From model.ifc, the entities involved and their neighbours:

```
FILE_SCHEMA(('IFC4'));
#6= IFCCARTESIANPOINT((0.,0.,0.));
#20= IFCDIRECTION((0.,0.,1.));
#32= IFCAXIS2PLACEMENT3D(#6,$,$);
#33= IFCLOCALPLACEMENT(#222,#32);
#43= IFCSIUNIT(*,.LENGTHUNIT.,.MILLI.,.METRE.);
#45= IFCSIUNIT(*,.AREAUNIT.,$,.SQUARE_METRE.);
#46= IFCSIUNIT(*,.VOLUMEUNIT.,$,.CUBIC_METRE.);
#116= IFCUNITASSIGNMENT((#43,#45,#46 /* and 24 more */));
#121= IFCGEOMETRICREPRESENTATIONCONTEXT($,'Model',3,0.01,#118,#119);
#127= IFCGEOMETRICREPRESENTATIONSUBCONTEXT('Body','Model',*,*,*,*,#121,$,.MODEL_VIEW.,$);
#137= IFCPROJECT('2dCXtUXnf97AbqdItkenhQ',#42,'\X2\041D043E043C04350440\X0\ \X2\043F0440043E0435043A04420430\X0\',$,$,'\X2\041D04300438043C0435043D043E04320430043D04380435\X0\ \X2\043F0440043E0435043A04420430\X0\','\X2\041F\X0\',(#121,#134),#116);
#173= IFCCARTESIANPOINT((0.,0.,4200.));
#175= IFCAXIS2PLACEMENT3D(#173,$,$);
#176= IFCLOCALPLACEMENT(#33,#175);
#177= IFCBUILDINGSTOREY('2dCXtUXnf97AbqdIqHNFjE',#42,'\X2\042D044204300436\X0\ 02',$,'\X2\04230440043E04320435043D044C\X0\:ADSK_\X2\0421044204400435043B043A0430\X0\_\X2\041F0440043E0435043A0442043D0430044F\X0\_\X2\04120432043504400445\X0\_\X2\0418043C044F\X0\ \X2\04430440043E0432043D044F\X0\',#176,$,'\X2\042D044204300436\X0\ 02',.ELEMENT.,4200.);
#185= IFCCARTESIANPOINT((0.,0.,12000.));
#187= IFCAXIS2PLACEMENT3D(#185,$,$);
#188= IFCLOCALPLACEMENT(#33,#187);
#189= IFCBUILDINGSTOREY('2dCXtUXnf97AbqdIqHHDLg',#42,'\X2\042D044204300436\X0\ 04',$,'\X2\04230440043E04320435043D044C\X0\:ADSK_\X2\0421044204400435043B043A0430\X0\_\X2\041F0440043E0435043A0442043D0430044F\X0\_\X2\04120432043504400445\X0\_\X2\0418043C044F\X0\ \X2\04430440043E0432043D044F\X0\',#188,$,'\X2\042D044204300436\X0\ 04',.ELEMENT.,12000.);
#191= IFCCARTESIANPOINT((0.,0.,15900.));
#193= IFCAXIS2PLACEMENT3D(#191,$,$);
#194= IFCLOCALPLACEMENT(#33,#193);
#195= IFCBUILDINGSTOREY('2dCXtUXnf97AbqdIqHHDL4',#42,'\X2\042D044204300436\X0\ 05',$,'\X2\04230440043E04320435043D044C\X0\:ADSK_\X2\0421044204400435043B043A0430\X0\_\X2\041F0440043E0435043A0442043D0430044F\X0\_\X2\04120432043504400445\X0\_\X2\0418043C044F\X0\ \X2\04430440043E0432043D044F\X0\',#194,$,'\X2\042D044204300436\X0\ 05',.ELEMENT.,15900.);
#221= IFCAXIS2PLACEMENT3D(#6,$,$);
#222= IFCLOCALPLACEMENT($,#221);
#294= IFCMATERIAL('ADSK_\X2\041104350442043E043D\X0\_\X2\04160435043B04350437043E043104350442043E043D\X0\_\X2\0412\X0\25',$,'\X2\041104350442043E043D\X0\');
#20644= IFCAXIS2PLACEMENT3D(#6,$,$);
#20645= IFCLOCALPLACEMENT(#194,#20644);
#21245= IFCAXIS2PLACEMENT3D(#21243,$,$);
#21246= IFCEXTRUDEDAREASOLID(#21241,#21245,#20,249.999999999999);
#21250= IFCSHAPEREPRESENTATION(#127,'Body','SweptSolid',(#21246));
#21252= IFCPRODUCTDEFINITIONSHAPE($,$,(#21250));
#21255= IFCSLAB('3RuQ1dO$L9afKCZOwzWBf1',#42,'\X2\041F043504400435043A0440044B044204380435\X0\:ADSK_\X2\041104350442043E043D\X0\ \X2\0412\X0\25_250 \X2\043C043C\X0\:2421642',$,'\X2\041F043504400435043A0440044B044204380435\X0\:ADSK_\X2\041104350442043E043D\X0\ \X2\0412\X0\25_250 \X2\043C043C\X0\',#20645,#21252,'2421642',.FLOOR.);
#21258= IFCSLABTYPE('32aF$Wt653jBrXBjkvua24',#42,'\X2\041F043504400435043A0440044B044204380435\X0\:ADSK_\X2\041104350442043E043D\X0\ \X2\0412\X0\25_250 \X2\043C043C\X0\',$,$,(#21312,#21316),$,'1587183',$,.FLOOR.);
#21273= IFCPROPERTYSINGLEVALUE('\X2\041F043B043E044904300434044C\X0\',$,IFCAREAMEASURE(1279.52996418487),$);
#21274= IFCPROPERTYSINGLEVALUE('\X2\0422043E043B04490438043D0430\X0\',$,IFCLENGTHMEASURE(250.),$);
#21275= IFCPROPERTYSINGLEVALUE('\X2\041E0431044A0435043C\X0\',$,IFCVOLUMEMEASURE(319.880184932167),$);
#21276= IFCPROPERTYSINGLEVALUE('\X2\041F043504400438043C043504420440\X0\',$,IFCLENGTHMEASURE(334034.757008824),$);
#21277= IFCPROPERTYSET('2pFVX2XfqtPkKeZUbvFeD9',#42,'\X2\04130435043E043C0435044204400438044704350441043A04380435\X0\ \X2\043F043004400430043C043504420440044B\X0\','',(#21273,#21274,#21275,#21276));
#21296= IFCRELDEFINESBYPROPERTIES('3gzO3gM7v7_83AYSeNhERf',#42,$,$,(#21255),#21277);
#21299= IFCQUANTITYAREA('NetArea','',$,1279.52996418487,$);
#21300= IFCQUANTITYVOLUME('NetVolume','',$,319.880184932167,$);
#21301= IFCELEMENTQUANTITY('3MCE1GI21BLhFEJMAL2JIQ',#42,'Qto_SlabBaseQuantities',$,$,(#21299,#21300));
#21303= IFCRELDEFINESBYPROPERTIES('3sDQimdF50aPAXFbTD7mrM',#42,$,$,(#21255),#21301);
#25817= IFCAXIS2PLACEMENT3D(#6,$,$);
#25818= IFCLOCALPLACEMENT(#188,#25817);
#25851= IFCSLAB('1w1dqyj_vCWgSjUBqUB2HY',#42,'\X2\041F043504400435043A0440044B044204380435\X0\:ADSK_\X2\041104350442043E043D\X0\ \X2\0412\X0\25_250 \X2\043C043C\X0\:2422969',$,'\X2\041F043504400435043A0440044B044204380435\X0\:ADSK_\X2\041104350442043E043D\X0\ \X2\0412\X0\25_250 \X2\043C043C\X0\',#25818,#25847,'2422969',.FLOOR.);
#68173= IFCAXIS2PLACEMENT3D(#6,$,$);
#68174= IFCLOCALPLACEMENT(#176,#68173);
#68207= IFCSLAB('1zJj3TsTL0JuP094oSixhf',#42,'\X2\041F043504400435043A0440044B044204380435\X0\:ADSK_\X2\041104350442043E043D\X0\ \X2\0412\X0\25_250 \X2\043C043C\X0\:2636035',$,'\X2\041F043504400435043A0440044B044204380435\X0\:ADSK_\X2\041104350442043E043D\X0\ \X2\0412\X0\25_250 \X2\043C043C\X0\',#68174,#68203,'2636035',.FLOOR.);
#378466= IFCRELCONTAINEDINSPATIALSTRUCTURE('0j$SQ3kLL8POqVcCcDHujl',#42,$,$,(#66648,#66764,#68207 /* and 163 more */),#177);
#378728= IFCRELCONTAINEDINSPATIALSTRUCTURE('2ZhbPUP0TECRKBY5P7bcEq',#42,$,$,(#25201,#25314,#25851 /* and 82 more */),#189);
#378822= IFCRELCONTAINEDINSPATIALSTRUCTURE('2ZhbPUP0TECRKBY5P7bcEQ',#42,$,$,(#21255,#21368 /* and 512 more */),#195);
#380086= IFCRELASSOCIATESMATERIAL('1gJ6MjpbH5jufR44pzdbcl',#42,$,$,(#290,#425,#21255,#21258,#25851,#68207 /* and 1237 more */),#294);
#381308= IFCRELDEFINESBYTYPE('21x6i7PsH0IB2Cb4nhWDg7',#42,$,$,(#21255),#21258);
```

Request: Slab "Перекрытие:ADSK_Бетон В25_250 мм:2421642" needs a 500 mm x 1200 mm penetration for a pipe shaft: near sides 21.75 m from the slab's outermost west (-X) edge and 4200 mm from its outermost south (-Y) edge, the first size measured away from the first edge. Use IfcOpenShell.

```python
import numpy as np
import ifcopenshell
import ifcopenshell.api.feature
import ifcopenshell.api.geometry
import ifcopenshell.api.pset
import ifcopenshell.api.root
import ifcopenshell.geom
import ifcopenshell.util.element
import ifcopenshell.util.placement
import ifcopenshell.util.representation
import ifcopenshell.util.shape
import ifcopenshell.util.unit

model = ifcopenshell.open("model.ifc")
unit_scale = ifcopenshell.util.unit.calculate_unit_scale(model)
area_scale = ifcopenshell.util.unit.calculate_unit_scale(model, "AREAUNIT")
volume_scale = ifcopenshell.util.unit.calculate_unit_scale(model, "VOLUMEUNIT")
settings = ifcopenshell.geom.settings()


def volume(element):
    """Net volume in cubic metres, openings subtracted."""
    shape = ifcopenshell.geom.create_shape(settings, element)
    return ifcopenshell.util.shape.get_volume(shape.geometry)


slab = model.by_guid("3RuQ1dO$L9afKCZOwzWBf1")
before = volume(slab)

# Extent in the slab's own axes, in metres. The edges named are its -X and -Y sides.
slab_shape = ifcopenshell.geom.create_shape(settings, slab)
vertices = ifcopenshell.util.shape.get_vertices(slab_shape.geometry)
x_min, y_min, bottom = vertices.min(axis=0)
top = vertices[:, 2].max()

opening = ifcopenshell.api.root.create_entity(model, ifc_class="IfcOpeningElement", name="Pipe shaft opening", predefined_type="OPENING")
context = ifcopenshell.util.representation.get_context(model, "Model", "Body", "MODEL_VIEW")
width, depth = 0.5, 1.2
outline = [(0.0, 0.0), (width, 0.0), (width, depth), (0.0, depth), (0.0, 0.0)]
# Overshoot both faces by 50 mm so the cut is clean.
shape = ifcopenshell.api.geometry.add_slab_representation(
    model, context=context, depth=top - bottom + 0.1, polyline=outline
)
ifcopenshell.api.geometry.assign_representation(model, product=opening, representation=shape)

matrix = ifcopenshell.util.placement.get_local_placement(slab.ObjectPlacement)
matrix[:, 3] = matrix @ np.append(np.array([x_min + 21.75, y_min + 4.2, bottom - 0.05]) / unit_scale, 1.0)
ifcopenshell.api.geometry.edit_object_placement(model, product=opening, matrix=matrix, is_si=False)
ifcopenshell.api.feature.add_feature(model, feature=opening, element=slab)

after = volume(slab)

# Update the slab's stored quantities.
pset = model.by_id(ifcopenshell.util.element.get_pset(slab, "Геометрические параметры", should_inherit=False)["id"])
ifcopenshell.api.pset.edit_pset(model, pset=pset, properties={
    "Площадь": model.create_entity("IfcAreaMeasure", after / (top - bottom) / area_scale),
    "Объем": model.create_entity("IfcVolumeMeasure", after / volume_scale),
})
qto = model.by_id(ifcopenshell.util.element.get_pset(slab, "Qto_SlabBaseQuantities", should_inherit=False)["id"])
ifcopenshell.api.pset.edit_qto(model, qto=qto, properties={
    "NetArea": after / (top - bottom) / area_scale,
    "NetVolume": after / volume_scale,
})

print(f"slab volume {before:.3f} -> {after:.3f} m3")

model.write("model_rev.ifc")
```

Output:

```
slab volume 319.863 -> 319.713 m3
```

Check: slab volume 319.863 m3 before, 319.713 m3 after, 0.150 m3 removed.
